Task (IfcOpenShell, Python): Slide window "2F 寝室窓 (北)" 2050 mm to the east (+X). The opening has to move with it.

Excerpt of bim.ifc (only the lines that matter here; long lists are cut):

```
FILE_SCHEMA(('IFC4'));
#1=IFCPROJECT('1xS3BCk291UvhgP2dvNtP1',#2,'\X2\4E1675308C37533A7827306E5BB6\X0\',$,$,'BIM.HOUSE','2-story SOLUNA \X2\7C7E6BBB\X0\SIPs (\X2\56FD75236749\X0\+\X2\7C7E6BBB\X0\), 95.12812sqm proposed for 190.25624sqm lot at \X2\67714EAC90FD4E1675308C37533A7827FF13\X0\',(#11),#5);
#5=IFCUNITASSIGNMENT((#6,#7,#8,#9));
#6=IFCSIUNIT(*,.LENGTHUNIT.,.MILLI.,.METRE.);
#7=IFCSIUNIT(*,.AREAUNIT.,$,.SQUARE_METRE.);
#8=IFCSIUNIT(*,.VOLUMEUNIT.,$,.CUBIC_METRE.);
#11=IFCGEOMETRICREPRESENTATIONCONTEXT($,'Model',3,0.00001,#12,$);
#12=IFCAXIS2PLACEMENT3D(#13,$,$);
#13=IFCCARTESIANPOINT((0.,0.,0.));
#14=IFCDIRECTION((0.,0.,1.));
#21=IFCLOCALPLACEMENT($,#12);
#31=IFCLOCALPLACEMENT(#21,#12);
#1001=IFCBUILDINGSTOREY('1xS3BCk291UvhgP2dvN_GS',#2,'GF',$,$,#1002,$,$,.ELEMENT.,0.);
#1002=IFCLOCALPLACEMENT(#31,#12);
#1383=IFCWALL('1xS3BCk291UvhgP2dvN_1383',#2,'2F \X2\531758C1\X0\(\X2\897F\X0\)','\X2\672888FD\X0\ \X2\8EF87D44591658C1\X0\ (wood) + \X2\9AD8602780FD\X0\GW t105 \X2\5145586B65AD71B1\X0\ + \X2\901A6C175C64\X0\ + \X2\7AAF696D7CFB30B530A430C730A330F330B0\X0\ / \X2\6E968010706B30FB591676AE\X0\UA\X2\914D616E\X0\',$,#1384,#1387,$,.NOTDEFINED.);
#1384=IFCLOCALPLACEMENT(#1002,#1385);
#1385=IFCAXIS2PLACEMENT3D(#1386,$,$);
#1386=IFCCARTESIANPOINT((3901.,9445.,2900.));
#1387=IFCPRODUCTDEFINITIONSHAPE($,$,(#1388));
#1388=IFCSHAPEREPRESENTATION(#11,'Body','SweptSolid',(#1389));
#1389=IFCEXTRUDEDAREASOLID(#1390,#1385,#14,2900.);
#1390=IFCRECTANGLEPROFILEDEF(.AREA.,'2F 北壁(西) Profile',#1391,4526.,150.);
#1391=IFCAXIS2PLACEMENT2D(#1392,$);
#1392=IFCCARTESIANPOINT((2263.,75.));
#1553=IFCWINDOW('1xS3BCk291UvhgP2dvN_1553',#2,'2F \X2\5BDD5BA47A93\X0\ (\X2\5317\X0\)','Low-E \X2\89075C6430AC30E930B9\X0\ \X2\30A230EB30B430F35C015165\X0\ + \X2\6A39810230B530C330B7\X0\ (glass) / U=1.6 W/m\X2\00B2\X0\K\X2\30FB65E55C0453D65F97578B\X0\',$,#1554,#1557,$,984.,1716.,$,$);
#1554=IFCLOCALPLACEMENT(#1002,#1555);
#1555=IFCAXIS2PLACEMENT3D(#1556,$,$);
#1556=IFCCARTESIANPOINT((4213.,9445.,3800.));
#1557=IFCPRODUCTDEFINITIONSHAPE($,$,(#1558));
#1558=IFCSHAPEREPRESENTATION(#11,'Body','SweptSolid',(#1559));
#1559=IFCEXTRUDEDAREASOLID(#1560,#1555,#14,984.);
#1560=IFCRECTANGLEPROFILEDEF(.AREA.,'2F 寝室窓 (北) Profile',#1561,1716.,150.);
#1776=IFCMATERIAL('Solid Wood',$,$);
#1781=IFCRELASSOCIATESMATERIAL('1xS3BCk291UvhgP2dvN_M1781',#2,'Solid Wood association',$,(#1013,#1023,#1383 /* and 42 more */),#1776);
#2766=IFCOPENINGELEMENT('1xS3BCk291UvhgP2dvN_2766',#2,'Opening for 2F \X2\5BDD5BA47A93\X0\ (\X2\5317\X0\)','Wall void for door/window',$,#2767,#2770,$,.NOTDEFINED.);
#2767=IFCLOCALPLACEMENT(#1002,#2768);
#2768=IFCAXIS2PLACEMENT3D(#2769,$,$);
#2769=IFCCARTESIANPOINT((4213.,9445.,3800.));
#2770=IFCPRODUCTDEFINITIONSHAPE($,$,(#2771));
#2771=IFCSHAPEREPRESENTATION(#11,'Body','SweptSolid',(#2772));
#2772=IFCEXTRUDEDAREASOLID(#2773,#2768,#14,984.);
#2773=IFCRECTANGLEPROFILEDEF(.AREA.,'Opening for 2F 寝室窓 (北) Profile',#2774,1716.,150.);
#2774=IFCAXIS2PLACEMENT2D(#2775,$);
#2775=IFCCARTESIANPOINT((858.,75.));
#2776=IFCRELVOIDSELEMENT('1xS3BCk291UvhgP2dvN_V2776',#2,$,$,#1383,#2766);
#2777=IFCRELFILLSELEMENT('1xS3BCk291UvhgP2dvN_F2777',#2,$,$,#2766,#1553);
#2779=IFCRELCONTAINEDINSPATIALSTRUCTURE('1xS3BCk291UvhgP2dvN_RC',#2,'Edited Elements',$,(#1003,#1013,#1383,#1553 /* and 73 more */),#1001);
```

```python
import ifcopenshell
import ifcopenshell.api.geometry
import ifcopenshell.util.placement

model = ifcopenshell.open("bim.ifc")

window = model.by_guid("1xS3BCk291UvhgP2dvN_1553")
opening = window.FillsVoids[0].RelatingOpeningElement
wall = opening.VoidsElements[0].RelatingBuildingElement

wall_matrix = ifcopenshell.util.placement.get_local_placement(wall.ObjectPlacement)
shift = wall_matrix[:3, 0] * 2050.0
before = ifcopenshell.util.placement.get_local_placement(window.ObjectPlacement)[:3, 3].copy()

# The window is not placed relative to its opening, so move both.
for product in (opening, window):
    matrix = ifcopenshell.util.placement.get_local_placement(product.ObjectPlacement)
    matrix[:3, 3] += shift
    ifcopenshell.api.geometry.edit_object_placement(model, product=product, matrix=matrix, is_si=False)

after = ifcopenshell.util.placement.get_local_placement(window.ObjectPlacement)[:3, 3]
print("window moved by", (after - before).round(3) + 0.0)

model.write("bim_v2.ifc")
```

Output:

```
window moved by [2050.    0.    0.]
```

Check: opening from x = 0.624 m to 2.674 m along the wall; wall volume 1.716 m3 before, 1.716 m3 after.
